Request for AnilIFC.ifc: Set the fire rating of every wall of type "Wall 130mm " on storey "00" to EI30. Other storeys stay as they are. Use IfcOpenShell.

First a look at what the model holds.

```python
import ifcopenshell
import ifcopenshell.util.element

model = ifcopenshell.open("AnilIFC.ifc")
print(model.schema)
storey = next(s for s in model.by_type("IfcBuildingStorey") if s.Name == "00")
walls = [e for e in ifcopenshell.util.element.get_decomposition(storey) if e.is_a("IfcWall")]
seen = {}
for e in walls:
    element_type = ifcopenshell.util.element.get_type(e)
    key = (element_type.Name if element_type != e and element_type else None, ifcopenshell.util.element.get_pset(e, "Pset_WallCommon", "FireRating"))
    seen[key] = seen.get(key, 0) + 1
for (name, value), count in sorted(seen.items(), key=str):
    print(count, "x", name, "|", value)
```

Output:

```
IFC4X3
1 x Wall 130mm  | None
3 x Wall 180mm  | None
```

```python
import ifcopenshell
import ifcopenshell.api.pset
import ifcopenshell.util.element

model = ifcopenshell.open("AnilIFC.ifc")

storey = next(s for s in model.by_type("IfcBuildingStorey") if s.Name == "00")
walls = [e for e in ifcopenshell.util.element.get_decomposition(storey) if e.is_a("IfcWall")]

count = 0
for e in walls:
    element_type = ifcopenshell.util.element.get_type(e)
    if element_type in (None, e) or element_type.Name != "Wall 130mm ":
        continue
    # add_pset returns the element's existing set when there is one.
    pset = ifcopenshell.api.pset.add_pset(model, product=e, name="Pset_WallCommon")
    ifcopenshell.api.pset.edit_pset(model, pset=pset, properties={"FireRating": "EI30"})
    count += 1

print(count, "walls updated")

model.write("AnilIFC-out.ifc")
```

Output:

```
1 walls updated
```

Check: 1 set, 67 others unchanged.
